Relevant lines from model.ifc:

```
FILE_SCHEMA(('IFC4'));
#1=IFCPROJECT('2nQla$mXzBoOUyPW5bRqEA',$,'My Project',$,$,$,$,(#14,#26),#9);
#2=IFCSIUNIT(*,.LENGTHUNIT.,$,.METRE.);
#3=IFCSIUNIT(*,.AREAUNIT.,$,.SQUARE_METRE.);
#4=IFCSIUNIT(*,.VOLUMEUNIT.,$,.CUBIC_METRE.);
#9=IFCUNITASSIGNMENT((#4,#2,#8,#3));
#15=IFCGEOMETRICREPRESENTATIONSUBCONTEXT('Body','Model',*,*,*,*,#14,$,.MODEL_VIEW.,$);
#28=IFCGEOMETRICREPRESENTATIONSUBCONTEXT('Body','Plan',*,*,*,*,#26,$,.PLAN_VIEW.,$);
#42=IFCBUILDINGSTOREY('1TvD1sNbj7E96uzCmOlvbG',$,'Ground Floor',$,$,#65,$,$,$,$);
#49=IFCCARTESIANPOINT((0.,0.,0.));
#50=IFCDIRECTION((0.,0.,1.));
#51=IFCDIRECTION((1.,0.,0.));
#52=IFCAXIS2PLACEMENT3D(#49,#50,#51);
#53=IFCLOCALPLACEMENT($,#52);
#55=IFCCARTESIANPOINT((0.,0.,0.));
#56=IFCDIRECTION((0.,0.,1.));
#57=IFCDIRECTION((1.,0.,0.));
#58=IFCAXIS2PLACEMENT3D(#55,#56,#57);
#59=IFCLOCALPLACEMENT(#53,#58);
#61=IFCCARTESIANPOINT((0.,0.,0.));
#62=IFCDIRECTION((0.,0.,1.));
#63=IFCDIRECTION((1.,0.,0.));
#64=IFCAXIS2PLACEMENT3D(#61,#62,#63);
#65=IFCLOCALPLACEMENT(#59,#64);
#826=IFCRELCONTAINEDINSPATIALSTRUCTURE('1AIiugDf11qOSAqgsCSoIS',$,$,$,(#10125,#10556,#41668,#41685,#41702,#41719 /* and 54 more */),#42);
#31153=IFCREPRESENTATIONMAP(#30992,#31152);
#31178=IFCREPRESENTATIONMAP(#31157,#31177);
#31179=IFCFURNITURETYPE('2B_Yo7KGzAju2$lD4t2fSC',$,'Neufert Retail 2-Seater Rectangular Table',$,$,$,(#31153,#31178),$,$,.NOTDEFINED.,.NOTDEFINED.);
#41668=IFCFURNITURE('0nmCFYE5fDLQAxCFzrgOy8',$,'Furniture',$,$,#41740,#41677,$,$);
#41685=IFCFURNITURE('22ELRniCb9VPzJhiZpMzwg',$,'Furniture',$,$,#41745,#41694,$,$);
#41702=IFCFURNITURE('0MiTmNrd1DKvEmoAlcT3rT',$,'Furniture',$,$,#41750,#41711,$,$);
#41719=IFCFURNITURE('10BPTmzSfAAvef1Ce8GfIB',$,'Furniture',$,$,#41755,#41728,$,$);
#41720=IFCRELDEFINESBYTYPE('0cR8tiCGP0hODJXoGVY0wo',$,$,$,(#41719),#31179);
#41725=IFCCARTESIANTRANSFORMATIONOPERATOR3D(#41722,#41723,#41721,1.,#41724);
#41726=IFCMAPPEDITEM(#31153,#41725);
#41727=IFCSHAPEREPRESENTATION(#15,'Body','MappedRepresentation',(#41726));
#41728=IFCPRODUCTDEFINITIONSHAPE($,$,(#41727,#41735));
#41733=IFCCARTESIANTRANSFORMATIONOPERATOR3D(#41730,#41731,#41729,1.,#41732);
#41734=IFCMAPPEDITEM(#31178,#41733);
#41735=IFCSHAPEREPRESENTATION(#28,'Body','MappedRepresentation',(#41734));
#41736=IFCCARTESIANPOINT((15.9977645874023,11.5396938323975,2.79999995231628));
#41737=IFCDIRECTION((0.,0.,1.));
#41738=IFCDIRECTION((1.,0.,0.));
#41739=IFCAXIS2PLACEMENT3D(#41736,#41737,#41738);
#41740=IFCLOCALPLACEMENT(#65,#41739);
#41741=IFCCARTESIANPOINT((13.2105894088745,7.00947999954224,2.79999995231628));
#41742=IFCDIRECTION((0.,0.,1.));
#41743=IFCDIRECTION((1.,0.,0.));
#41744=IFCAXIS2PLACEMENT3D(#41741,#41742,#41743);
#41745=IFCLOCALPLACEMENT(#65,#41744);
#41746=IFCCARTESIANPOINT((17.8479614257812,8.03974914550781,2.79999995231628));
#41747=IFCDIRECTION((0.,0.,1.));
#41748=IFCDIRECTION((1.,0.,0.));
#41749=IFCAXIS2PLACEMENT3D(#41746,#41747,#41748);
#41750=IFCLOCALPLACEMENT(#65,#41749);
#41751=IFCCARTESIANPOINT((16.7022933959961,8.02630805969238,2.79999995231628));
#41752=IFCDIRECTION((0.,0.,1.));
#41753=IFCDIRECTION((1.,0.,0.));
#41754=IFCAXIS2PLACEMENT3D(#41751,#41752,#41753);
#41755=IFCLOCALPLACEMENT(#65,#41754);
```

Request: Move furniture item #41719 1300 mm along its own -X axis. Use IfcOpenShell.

```python
import ifcopenshell
import ifcopenshell.api.geometry
import ifcopenshell.util.placement

model = ifcopenshell.open("model.ifc")

item = model.by_guid("10BPTmzSfAAvef1Ce8GfIB")
matrix = ifcopenshell.util.placement.get_local_placement(item.ObjectPlacement)
matrix[:3, 3] -= matrix[:3, 0] * 1.3
ifcopenshell.api.geometry.edit_object_placement(model, product=item, matrix=matrix, is_si=False)

print(ifcopenshell.util.placement.get_local_placement(item.ObjectPlacement).round(3) + 0.0)

model.write("model_rev.ifc")
```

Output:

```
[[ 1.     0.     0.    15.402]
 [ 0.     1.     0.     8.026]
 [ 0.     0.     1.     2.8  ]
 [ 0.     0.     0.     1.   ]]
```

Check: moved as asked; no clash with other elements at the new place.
